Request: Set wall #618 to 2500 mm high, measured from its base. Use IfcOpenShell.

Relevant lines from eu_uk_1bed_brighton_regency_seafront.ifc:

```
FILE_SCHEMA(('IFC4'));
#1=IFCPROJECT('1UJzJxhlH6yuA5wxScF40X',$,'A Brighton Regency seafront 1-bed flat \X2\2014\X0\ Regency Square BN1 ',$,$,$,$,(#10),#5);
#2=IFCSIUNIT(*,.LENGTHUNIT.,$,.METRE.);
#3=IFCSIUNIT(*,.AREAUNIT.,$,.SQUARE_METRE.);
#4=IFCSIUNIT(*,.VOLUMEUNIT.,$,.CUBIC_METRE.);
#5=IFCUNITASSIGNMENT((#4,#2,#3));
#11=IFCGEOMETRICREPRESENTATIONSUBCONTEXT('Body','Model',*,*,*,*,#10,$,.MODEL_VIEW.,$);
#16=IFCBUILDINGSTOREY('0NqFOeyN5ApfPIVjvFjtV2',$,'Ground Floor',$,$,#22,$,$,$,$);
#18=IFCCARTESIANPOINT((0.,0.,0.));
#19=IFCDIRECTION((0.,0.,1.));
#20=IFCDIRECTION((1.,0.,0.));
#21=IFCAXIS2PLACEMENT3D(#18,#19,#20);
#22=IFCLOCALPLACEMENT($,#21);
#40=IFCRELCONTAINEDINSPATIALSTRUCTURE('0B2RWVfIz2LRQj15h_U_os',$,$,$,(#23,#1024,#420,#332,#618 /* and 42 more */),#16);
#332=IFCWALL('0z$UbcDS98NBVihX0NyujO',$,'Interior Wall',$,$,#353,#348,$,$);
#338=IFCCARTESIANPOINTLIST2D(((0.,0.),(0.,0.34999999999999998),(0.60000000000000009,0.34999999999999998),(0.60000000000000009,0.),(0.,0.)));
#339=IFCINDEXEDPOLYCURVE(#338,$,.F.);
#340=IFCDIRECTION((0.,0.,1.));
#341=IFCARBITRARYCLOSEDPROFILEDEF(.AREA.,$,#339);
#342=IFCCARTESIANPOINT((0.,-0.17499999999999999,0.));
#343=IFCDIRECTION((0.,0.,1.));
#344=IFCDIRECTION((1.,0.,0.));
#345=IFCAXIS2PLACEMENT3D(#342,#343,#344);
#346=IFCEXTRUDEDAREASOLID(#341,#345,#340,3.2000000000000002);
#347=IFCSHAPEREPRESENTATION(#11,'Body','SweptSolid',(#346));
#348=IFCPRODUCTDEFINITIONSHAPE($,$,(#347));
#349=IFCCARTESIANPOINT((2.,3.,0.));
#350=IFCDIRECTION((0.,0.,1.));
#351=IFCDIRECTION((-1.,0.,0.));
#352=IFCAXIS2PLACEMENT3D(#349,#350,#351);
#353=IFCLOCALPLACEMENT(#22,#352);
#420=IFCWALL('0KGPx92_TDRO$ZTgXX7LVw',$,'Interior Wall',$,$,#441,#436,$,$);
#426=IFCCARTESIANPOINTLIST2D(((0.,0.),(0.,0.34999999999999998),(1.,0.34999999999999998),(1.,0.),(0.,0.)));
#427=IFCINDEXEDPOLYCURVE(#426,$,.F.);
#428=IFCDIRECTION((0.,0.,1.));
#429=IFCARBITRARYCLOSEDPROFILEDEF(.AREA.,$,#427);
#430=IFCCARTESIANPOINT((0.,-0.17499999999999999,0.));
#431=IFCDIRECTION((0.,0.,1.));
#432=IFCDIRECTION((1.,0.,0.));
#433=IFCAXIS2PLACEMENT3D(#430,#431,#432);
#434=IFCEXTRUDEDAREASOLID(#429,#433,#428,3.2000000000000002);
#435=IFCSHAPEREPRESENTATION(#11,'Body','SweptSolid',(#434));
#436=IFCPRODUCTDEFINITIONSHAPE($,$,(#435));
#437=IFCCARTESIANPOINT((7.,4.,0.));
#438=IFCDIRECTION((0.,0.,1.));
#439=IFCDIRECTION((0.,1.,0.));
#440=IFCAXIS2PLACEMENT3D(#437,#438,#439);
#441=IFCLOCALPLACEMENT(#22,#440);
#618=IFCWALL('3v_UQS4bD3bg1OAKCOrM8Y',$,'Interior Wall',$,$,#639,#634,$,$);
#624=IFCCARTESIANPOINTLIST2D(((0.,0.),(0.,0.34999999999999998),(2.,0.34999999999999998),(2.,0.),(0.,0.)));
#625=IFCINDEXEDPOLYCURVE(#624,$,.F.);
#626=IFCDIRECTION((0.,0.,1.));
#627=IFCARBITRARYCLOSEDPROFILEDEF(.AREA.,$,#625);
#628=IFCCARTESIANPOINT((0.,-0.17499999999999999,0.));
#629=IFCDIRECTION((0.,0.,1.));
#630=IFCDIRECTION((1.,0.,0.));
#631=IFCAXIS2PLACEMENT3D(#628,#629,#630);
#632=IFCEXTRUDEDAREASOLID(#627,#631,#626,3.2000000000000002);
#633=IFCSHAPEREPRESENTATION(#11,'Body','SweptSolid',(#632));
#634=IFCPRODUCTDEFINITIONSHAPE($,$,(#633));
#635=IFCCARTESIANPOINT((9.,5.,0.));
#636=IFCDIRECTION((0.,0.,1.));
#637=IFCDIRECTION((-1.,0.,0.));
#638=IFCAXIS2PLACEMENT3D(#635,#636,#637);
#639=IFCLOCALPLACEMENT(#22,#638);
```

```python
import ifcopenshell
import ifcopenshell.geom
import ifcopenshell.util.representation
import ifcopenshell.util.shape
import ifcopenshell.util.unit

model = ifcopenshell.open("eu_uk_1bed_brighton_regency_seafront.ifc")
unit_scale = ifcopenshell.util.unit.calculate_unit_scale(model)
settings = ifcopenshell.geom.settings()


def volume(element):
    """Net volume in cubic metres, openings subtracted."""
    shape = ifcopenshell.geom.create_shape(settings, element)
    return ifcopenshell.util.shape.get_volume(shape.geometry)


wall = model.by_guid("3v_UQS4bD3bg1OAKCOrM8Y")
before = volume(wall)

body = ifcopenshell.util.representation.get_representation(wall, "Model", "Body")
solid = body.Items[0]
old_height = solid.Depth
solid.Depth = 2.5 / unit_scale
after = volume(wall)

print(f"height {old_height:g} -> {solid.Depth:g}, volume {before:.3f} -> {after:.3f} m3")

model.write("eu_uk_1bed_brighton_regency_seafront_updated.ifc")
```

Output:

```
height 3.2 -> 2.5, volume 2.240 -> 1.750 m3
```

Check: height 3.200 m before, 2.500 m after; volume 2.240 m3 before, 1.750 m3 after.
